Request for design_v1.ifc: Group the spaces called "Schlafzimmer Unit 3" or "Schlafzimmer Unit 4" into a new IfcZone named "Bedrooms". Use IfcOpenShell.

First a look at what the model holds.

```python
import ifcopenshell

model = ifcopenshell.open("design_v1.ifc")
print(model.schema)
seen = {}
for space in model.by_type("IfcSpace"):
    seen[space.LongName] = seen.get(space.LongName, 0) + 1
for name, count in sorted(seen.items(), key=str):
    print(count, "x", name)
print("zones:", [z.Name for z in model.by_type("IfcZone")][:20])
```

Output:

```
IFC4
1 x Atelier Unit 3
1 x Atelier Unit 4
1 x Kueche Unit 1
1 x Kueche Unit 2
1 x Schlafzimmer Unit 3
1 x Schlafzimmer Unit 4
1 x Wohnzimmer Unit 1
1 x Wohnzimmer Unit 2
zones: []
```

```python
import ifcopenshell
import ifcopenshell.api.group
import ifcopenshell.api.root

model = ifcopenshell.open("design_v1.ifc")

names = {"Schlafzimmer Unit 3", "Schlafzimmer Unit 4"}
spaces = [s for s in model.by_type("IfcSpace") if s.LongName in names]

zone = ifcopenshell.api.root.create_entity(model, ifc_class="IfcZone", name="Bedrooms")
ifcopenshell.api.group.assign_group(model, products=spaces, group=zone)
print(len(spaces), "spaces in", zone.Name)

model.write("design_v1_edited.ifc")
```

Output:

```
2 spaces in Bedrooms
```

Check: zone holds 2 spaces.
